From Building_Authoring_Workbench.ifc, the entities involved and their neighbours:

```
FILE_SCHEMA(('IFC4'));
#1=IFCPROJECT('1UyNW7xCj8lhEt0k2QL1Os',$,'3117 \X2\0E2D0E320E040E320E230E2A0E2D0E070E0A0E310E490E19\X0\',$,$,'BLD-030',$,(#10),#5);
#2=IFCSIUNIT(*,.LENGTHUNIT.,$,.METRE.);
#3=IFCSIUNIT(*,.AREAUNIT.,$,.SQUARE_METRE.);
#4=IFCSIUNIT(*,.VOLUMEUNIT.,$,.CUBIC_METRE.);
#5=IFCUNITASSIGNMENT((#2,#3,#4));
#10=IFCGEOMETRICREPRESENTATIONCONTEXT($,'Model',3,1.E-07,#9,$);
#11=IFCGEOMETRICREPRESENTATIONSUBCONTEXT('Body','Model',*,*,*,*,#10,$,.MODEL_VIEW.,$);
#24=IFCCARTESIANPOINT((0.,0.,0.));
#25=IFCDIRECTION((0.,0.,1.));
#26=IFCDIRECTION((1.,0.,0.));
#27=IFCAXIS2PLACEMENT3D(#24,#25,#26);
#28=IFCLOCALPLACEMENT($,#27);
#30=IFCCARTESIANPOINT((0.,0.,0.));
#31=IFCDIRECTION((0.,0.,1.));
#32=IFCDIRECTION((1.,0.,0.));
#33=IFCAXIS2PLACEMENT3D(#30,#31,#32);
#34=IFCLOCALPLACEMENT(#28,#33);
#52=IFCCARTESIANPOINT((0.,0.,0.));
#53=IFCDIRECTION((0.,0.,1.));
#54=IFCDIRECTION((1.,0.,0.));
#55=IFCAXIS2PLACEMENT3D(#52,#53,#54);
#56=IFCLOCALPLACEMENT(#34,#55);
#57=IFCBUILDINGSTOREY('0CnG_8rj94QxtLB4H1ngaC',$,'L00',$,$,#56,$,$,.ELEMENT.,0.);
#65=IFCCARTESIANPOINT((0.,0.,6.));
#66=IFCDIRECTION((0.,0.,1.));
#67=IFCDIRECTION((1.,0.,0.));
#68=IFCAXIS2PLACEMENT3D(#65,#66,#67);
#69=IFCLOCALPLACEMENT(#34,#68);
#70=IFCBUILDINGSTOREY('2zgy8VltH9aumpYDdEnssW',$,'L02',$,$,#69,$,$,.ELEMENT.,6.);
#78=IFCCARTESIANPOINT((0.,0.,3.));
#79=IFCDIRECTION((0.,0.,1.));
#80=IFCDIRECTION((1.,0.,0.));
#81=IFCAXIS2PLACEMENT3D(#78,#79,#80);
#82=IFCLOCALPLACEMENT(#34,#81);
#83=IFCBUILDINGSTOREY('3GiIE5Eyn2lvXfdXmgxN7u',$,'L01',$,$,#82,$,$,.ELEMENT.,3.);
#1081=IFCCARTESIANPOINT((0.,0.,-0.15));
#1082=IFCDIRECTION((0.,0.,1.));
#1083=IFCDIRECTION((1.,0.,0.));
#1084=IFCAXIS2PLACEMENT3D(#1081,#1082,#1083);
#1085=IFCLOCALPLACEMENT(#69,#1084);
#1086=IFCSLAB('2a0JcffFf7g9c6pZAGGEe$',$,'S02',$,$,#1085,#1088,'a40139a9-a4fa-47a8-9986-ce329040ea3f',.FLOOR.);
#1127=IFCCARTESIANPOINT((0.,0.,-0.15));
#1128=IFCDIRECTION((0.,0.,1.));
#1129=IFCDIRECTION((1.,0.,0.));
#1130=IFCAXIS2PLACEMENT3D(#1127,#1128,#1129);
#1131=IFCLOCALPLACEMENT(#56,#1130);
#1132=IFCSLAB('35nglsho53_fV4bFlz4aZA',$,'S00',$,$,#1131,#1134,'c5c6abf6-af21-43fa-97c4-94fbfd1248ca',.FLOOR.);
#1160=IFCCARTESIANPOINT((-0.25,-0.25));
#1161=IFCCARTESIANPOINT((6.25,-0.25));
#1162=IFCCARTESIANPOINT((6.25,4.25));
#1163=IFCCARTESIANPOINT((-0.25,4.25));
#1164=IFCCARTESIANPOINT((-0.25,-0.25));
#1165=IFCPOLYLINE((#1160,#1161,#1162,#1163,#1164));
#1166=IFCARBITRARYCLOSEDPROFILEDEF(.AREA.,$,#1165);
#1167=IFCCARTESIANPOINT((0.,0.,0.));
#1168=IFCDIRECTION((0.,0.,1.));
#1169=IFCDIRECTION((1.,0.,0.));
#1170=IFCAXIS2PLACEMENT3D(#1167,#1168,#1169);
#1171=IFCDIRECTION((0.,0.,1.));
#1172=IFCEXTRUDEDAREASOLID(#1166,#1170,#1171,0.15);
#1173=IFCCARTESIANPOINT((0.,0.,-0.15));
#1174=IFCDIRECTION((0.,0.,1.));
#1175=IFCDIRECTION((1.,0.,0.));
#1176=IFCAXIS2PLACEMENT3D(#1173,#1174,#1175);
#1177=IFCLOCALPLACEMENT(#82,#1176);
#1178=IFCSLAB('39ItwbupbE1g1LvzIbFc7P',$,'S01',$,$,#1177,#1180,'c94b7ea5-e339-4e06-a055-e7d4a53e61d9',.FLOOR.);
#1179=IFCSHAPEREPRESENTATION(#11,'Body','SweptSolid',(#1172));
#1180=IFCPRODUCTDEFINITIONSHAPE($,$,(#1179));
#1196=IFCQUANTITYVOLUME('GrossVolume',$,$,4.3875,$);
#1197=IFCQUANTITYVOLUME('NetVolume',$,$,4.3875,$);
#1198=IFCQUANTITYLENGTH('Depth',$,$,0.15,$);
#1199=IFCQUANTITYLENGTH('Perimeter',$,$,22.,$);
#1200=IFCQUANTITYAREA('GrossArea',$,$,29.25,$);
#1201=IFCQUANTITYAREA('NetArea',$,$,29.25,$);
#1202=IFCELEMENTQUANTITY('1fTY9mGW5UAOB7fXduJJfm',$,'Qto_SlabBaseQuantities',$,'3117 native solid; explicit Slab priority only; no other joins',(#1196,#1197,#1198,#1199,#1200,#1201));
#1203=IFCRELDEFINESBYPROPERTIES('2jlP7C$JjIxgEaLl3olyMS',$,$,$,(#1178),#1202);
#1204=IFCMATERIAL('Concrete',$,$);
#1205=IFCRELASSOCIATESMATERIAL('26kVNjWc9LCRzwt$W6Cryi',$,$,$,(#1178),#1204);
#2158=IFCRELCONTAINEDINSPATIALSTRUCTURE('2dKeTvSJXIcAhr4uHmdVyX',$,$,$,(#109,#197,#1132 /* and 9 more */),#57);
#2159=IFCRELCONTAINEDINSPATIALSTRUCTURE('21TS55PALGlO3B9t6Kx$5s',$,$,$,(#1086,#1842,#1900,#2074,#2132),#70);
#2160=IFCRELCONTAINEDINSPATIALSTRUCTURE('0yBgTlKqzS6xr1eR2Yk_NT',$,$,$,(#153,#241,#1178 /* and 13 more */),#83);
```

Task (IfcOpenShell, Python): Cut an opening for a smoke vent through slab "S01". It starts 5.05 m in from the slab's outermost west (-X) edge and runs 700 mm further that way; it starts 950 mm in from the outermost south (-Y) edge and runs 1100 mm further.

```python
import numpy as np
import ifcopenshell
import ifcopenshell.api.feature
import ifcopenshell.api.geometry
import ifcopenshell.api.pset
import ifcopenshell.api.root
import ifcopenshell.geom
import ifcopenshell.util.element
import ifcopenshell.util.placement
import ifcopenshell.util.representation
import ifcopenshell.util.shape
import ifcopenshell.util.unit

model = ifcopenshell.open("Building_Authoring_Workbench.ifc")
unit_scale = ifcopenshell.util.unit.calculate_unit_scale(model)
area_scale = ifcopenshell.util.unit.calculate_unit_scale(model, "AREAUNIT")
volume_scale = ifcopenshell.util.unit.calculate_unit_scale(model, "VOLUMEUNIT")
settings = ifcopenshell.geom.settings()


def volume(element):
    """Net volume in cubic metres, openings subtracted."""
    shape = ifcopenshell.geom.create_shape(settings, element)
    return ifcopenshell.util.shape.get_volume(shape.geometry)


slab = model.by_guid("39ItwbupbE1g1LvzIbFc7P")
before = volume(slab)

# Extent in the slab's own axes, in metres. The edges named are its -X and -Y sides.
slab_shape = ifcopenshell.geom.create_shape(settings, slab)
vertices = ifcopenshell.util.shape.get_vertices(slab_shape.geometry)
x_min, y_min, bottom = vertices.min(axis=0)
top = vertices[:, 2].max()

opening = ifcopenshell.api.root.create_entity(model, ifc_class="IfcOpeningElement", name="Smoke vent opening", predefined_type="OPENING")
context = ifcopenshell.util.representation.get_context(model, "Model", "Body", "MODEL_VIEW")
width, depth = 0.7, 1.1
outline = [(0.0, 0.0), (width, 0.0), (width, depth), (0.0, depth), (0.0, 0.0)]
# Overshoot both faces by 50 mm so the cut is clean.
shape = ifcopenshell.api.geometry.add_slab_representation(
    model, context=context, depth=top - bottom + 0.1, polyline=outline
)
ifcopenshell.api.geometry.assign_representation(model, product=opening, representation=shape)

matrix = ifcopenshell.util.placement.get_local_placement(slab.ObjectPlacement)
matrix[:, 3] = matrix @ np.append(np.array([x_min + 5.05, y_min + 0.95, bottom - 0.05]) / unit_scale, 1.0)
ifcopenshell.api.geometry.edit_object_placement(model, product=opening, matrix=matrix, is_si=False)
ifcopenshell.api.feature.add_feature(model, feature=opening, element=slab)

after = volume(slab)

# Update the slab's stored quantities.
qto = model.by_id(ifcopenshell.util.element.get_pset(slab, "Qto_SlabBaseQuantities", should_inherit=False)["id"])
ifcopenshell.api.pset.edit_qto(model, qto=qto, properties={
    "NetVolume": after / volume_scale,
    "NetArea": after / (top - bottom) / area_scale,
})

print(f"slab volume {before:.3f} -> {after:.3f} m3")

model.write("Building_Authoring_Workbench-out.ifc")
```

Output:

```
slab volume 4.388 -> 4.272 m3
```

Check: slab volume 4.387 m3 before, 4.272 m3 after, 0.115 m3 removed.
